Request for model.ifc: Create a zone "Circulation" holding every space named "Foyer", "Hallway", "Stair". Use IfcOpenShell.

First a look at what the model holds.

```python
import ifcopenshell

model = ifcopenshell.open("model.ifc")
print(model.schema)
seen = {}
for space in model.by_type("IfcSpace"):
    seen[space.LongName] = seen.get(space.LongName, 0) + 1
for name, count in sorted(seen.items(), key=str):
    print(count, "x", name)
print("zones:", [z.Name for z in model.by_type("IfcZone")][:20])
```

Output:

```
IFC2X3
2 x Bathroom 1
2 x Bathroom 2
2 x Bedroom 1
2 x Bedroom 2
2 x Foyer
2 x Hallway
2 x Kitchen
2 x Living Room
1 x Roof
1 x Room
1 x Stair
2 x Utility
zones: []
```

```python
import ifcopenshell
import ifcopenshell.api.group
import ifcopenshell.api.root

model = ifcopenshell.open("model.ifc")

names = {"Foyer", "Hallway", "Stair"}
spaces = [s for s in model.by_type("IfcSpace") if s.LongName in names]

zone = ifcopenshell.api.root.create_entity(model, ifc_class="IfcZone", name="Circulation")
ifcopenshell.api.group.assign_group(model, products=spaces, group=zone)
print(len(spaces), "spaces in", zone.Name)

model.write("model_updated.ifc")
```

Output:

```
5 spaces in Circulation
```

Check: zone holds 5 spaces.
